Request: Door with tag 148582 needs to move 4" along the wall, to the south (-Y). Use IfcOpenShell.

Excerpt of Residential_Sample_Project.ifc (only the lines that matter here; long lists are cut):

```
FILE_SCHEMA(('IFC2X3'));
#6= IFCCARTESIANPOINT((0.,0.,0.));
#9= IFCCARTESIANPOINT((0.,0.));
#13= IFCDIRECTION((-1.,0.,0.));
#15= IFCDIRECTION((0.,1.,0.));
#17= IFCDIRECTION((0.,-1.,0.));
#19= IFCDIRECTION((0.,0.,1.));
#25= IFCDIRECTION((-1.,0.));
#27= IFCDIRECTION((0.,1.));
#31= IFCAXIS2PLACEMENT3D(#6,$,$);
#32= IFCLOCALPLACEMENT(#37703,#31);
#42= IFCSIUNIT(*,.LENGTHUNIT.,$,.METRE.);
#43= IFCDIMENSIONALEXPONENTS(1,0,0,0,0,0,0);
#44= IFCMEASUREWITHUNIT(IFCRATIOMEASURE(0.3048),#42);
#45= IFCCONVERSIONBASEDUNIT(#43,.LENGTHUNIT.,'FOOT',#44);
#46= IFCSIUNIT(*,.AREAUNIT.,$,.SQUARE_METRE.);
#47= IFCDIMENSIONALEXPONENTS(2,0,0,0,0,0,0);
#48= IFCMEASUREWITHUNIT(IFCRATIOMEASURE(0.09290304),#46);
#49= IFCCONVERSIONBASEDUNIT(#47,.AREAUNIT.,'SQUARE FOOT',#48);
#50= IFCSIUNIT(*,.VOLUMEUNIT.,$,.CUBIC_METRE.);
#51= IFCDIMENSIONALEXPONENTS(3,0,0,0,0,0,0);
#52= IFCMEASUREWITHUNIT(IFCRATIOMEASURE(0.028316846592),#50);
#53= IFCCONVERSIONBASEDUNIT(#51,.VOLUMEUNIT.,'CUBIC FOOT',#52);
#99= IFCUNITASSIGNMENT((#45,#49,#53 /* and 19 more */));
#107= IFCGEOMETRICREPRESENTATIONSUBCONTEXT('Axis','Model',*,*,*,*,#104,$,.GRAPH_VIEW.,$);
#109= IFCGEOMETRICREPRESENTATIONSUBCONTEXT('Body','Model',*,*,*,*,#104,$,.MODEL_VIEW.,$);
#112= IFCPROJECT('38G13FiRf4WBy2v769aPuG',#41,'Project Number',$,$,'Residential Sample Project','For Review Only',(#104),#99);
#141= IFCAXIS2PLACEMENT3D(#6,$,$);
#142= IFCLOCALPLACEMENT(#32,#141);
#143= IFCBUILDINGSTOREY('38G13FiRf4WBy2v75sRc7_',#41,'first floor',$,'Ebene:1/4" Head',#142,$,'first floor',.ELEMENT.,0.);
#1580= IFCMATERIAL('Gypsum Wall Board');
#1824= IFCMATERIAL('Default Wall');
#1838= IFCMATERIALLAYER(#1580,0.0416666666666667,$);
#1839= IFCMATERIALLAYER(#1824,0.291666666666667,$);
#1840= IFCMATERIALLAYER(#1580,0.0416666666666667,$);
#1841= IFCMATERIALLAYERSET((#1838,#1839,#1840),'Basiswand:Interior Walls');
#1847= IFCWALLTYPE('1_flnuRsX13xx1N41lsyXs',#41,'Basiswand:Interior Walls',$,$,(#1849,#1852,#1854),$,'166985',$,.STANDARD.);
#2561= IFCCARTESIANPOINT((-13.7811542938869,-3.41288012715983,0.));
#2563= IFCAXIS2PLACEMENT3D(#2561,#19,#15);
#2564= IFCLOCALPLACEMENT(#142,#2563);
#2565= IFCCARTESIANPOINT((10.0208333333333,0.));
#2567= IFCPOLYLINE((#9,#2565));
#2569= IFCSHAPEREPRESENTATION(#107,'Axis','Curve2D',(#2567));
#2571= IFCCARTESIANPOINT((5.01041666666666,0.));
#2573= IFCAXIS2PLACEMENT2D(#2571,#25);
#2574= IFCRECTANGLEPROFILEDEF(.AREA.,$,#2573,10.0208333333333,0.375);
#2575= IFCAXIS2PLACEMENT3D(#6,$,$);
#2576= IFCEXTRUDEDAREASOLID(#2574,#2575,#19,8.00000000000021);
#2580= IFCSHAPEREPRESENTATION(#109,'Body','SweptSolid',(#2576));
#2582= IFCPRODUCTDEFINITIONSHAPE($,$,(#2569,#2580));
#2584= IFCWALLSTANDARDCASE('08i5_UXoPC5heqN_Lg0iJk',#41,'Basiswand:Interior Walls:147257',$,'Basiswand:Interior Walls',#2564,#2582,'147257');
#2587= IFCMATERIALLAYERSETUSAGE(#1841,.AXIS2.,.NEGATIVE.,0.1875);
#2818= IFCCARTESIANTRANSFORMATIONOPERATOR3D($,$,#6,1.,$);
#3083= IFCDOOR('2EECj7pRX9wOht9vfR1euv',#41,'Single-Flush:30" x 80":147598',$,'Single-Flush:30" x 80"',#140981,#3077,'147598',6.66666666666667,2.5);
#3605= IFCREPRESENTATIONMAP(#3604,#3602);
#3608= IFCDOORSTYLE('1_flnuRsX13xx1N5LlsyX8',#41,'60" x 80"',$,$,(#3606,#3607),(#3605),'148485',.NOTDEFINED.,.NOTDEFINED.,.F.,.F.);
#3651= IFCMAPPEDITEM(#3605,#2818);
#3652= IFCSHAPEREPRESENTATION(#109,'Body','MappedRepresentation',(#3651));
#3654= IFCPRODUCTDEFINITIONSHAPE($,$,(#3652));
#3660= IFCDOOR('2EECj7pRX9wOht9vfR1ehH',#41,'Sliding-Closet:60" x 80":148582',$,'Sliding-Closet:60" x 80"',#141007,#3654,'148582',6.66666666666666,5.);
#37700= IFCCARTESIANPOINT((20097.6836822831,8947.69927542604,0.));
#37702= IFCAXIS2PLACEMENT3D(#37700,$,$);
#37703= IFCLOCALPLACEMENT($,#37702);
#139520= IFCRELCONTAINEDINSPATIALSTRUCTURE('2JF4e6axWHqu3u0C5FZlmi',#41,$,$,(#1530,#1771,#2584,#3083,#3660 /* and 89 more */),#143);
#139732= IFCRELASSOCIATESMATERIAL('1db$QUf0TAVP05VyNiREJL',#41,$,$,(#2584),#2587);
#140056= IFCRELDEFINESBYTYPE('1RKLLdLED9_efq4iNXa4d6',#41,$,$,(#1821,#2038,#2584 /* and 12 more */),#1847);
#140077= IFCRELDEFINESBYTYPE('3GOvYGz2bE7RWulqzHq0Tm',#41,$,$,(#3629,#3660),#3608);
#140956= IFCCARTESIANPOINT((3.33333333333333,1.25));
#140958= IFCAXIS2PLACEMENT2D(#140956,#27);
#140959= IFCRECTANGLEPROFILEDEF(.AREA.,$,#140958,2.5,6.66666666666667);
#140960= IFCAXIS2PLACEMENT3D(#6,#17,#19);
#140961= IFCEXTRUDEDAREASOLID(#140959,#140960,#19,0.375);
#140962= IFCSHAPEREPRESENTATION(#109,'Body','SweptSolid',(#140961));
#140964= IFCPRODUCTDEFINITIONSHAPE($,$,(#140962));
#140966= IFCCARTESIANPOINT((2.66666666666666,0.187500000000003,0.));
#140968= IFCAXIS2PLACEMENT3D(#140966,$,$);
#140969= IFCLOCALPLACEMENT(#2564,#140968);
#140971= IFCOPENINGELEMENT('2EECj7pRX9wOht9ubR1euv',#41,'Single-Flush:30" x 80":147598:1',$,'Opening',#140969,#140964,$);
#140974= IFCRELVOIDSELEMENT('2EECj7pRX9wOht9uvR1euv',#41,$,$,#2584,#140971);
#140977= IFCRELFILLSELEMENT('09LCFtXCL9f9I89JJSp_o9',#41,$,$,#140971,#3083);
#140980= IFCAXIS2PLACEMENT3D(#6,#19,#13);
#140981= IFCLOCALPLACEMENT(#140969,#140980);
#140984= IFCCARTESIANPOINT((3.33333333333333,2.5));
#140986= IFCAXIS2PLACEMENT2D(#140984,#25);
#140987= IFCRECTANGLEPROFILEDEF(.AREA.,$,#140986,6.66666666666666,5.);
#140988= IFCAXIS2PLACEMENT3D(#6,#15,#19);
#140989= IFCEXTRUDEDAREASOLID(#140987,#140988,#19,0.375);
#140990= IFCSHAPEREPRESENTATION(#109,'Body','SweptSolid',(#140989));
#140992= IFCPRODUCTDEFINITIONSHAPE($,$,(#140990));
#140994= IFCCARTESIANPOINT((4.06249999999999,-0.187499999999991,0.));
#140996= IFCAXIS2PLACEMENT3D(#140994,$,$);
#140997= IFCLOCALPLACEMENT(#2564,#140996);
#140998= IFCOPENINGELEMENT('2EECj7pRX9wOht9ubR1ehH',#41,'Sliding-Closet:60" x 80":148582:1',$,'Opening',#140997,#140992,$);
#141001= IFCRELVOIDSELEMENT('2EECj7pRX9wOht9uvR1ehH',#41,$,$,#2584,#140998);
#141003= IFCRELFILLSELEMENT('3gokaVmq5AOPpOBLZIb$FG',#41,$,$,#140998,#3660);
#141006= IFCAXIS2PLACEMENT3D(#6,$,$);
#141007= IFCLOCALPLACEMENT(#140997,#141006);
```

```python
import ifcopenshell
import ifcopenshell.api.geometry
import ifcopenshell.util.placement
import ifcopenshell.util.unit

model = ifcopenshell.open("Residential_Sample_Project.ifc")
unit_scale = ifcopenshell.util.unit.calculate_unit_scale(model)

door = model.by_id(3660)
opening = door.FillsVoids[0].RelatingOpeningElement
wall = opening.VoidsElements[0].RelatingBuildingElement

wall_matrix = ifcopenshell.util.placement.get_local_placement(wall.ObjectPlacement)
shift = wall_matrix[:3, 0] * -4 * 0.0254 / unit_scale
before = ifcopenshell.util.placement.get_local_placement(door.ObjectPlacement)[:3, 3].copy()

# The door is placed relative to its opening, so it follows when the opening moves.
matrix = ifcopenshell.util.placement.get_local_placement(opening.ObjectPlacement)
matrix[:3, 3] += shift
ifcopenshell.api.geometry.edit_object_placement(
    model, product=opening, matrix=matrix, is_si=False, should_transform_children=True
)

after = ifcopenshell.util.placement.get_local_placement(door.ObjectPlacement)[:3, 3]
print("door moved by", (after - before).round(3) + 0.0)

model.write("Residential_Sample_Project_edited.ifc")
```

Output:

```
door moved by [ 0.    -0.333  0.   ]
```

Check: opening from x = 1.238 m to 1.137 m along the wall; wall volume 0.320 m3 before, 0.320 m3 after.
